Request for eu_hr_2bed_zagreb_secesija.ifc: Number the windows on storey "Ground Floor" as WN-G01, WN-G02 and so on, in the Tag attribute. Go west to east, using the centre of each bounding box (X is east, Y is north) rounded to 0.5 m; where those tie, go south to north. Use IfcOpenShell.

First a look at what the model holds.

```python
import ifcopenshell
import ifcopenshell.util.element
import ifcopenshell.util.placement

model = ifcopenshell.open("eu_hr_2bed_zagreb_secesija.ifc")
print(model.schema)
storey = next(s for s in model.by_type("IfcBuildingStorey") if s.Name == "Ground Floor")
windows = [e for e in ifcopenshell.util.element.get_decomposition(storey) if e.is_a("IfcWindow")]
for e in sorted(windows, key=lambda e: e.id()):
    origin = ifcopenshell.util.placement.get_local_placement(e.ObjectPlacement)[:3, 3]
    print(e.id(), e.Tag, e.Name, origin.round(2) + 0.0, sep=" | ")
```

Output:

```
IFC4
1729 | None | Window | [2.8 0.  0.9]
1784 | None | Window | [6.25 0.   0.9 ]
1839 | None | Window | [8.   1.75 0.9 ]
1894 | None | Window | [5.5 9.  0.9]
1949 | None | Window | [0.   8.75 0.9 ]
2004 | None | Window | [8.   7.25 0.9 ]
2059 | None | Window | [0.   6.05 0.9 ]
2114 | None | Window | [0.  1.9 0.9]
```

```python
import ifcopenshell
import ifcopenshell.geom
import ifcopenshell.util.element
import ifcopenshell.util.shape

model = ifcopenshell.open("eu_hr_2bed_zagreb_secesija.ifc")
settings = ifcopenshell.geom.settings()
settings.set("use-world-coords", True)


def centre(element):
    shape = ifcopenshell.geom.create_shape(settings, element)
    return ifcopenshell.util.shape.get_bbox_centroid(shape.geometry)


storey = next(s for s in model.by_type("IfcBuildingStorey") if s.Name == "Ground Floor")
windows = [e for e in ifcopenshell.util.element.get_decomposition(storey) if e.is_a("IfcWindow")]

# Insertion points can sit at a corner or the storey origin, so sort by the geometry (in metres).
centres = {e: centre(e) for e in windows}
windows.sort(key=lambda e: (round(centres[e][0] / 0.5), centres[e][1]))

for i, e in enumerate(windows, start=1):
    number = f"WN-G{i:02d}"
    e.Tag = number
    print(e.id(), number)

model.write("eu_hr_2bed_zagreb_secesija_v2.ifc")
```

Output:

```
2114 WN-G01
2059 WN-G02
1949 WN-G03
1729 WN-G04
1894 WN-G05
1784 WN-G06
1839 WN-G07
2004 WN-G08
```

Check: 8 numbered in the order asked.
